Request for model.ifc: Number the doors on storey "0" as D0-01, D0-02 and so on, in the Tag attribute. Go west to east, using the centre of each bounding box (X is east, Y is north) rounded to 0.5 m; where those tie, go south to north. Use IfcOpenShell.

First a look at what the model holds.

```python
import ifcopenshell
import ifcopenshell.util.element
import ifcopenshell.util.placement

model = ifcopenshell.open("model.ifc")
print(model.schema)
storey = next(s for s in model.by_type("IfcBuildingStorey") if s.Name == "0")
doors = [e for e in ifcopenshell.util.element.get_decomposition(storey) if e.is_a("IfcDoor")]
for e in sorted(doors, key=lambda e: e.id()):
    origin = ifcopenshell.util.placement.get_local_placement(e.ObjectPlacement)[:3, 3]
    print(e.id(), e.Tag, e.Name, origin.round(2) + 0.0, sep=" | ")
```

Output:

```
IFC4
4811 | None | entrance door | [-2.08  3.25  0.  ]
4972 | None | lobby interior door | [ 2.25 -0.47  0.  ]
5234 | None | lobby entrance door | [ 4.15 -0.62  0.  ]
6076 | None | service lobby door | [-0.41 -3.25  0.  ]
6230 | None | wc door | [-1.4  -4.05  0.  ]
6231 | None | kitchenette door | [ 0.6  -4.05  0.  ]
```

```python
import ifcopenshell
import ifcopenshell.geom
import ifcopenshell.util.element
import ifcopenshell.util.shape

model = ifcopenshell.open("model.ifc")
settings = ifcopenshell.geom.settings()
settings.set("use-world-coords", True)


def centre(element):
    shape = ifcopenshell.geom.create_shape(settings, element)
    return ifcopenshell.util.shape.get_bbox_centroid(shape.geometry)


storey = next(s for s in model.by_type("IfcBuildingStorey") if s.Name == "0")
doors = [e for e in ifcopenshell.util.element.get_decomposition(storey) if e.is_a("IfcDoor")]

# Insertion points can sit at a corner or the storey origin, so sort by the geometry (in metres).
centres = {e: centre(e) for e in doors}
doors.sort(key=lambda e: (round(centres[e][0] / 0.5), centres[e][1]))

for i, e in enumerate(doors, start=1):
    number = f"D0-{i:02d}"
    e.Tag = number
    print(e.id(), number)

model.write("model-out.ifc")
```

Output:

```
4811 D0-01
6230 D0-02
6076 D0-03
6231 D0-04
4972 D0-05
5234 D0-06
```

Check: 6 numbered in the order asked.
